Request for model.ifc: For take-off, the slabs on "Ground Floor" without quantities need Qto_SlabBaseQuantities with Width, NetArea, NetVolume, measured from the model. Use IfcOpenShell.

First a look at what the model holds.

```python
import ifcopenshell
import ifcopenshell.util.element
import ifcopenshell.util.unit

model = ifcopenshell.open("model.ifc")
print(model.schema)
for unit_type in ("LENGTHUNIT", "AREAUNIT", "VOLUMEUNIT"):
    print(unit_type, ifcopenshell.util.unit.calculate_unit_scale(model, unit_type))
storey = next(s for s in model.by_type("IfcBuildingStorey") if s.Name == "Ground Floor")
slabs = [e for e in ifcopenshell.util.element.get_decomposition(storey) if e.is_a("IfcSlab")]
for e in sorted(slabs, key=lambda e: e.id()):
    print(e.id(), e.is_a(), e.Name, list(ifcopenshell.util.element.get_psets(e, qtos_only=True)), sep=" | ")
```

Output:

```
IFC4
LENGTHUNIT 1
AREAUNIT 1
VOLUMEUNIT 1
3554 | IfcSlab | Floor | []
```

```python
import ifcopenshell
import ifcopenshell.api.pset
import ifcopenshell.geom
import ifcopenshell.util.element
import ifcopenshell.util.shape
import ifcopenshell.util.unit

model = ifcopenshell.open("model.ifc")
unit_scale = ifcopenshell.util.unit.calculate_unit_scale(model)
area_scale = ifcopenshell.util.unit.calculate_unit_scale(model, "AREAUNIT")
volume_scale = ifcopenshell.util.unit.calculate_unit_scale(model, "VOLUMEUNIT")
settings = ifcopenshell.geom.settings()

storey = next(s for s in model.by_type("IfcBuildingStorey") if s.Name == "Ground Floor")
slabs = [e for e in ifcopenshell.util.element.get_decomposition(storey) if e.is_a("IfcSlab")]

for e in sorted(slabs, key=lambda e: e.id()):
    if ifcopenshell.util.element.get_psets(e, qtos_only=True, should_inherit=False):
        continue
    # Geometry comes back in metres, in the element's own axes.
    shape = ifcopenshell.geom.create_shape(settings, e)
    values = {
        "Width": ifcopenshell.util.shape.get_z(shape.geometry) / unit_scale,
        "NetArea": ifcopenshell.util.shape.get_footprint_area(shape.geometry) / area_scale,
        "NetVolume": ifcopenshell.util.shape.get_volume(shape.geometry) / volume_scale,
    }
    qto = ifcopenshell.api.pset.add_qto(model, product=e, name="Qto_SlabBaseQuantities")
    ifcopenshell.api.pset.edit_qto(model, qto=qto, properties=values)
    print(e.id(), {k: round(v, 3) for k, v in values.items()})

model.write("model_edited.ifc")
```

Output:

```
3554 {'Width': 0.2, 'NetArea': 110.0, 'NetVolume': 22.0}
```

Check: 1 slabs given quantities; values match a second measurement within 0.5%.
